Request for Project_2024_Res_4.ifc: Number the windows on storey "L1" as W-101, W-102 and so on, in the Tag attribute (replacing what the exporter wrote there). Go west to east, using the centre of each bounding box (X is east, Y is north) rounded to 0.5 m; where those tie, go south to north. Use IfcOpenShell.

First a look at what the model holds.

```python
import ifcopenshell
import ifcopenshell.util.element
import ifcopenshell.util.placement

model = ifcopenshell.open("Project_2024_Res_4.ifc")
print(model.schema)
storey = next(s for s in model.by_type("IfcBuildingStorey") if s.Name == "L1")
windows = [e for e in ifcopenshell.util.element.get_decomposition(storey) if e.is_a("IfcWindow")]
for e in sorted(windows, key=lambda e: e.id()):
    origin = ifcopenshell.util.placement.get_local_placement(e.ObjectPlacement)[:3, 3]
    print(e.id(), e.Tag, e.Name, origin.round(2) + 0.0, sep=" | ")
```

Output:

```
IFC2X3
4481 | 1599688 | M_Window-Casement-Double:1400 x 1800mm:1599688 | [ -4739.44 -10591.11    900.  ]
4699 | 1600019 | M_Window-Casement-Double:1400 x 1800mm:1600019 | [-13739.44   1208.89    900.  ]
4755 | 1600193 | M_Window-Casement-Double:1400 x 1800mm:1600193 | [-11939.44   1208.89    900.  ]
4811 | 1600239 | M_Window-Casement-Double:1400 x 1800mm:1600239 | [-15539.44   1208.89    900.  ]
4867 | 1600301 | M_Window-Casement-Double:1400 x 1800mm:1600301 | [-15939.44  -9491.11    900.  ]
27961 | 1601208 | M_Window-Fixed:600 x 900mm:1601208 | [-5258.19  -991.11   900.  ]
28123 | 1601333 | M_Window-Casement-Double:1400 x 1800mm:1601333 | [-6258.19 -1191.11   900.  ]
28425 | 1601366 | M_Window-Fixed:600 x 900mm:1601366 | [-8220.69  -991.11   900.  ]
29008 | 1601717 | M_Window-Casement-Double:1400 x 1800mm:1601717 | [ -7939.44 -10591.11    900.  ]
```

```python
import ifcopenshell
import ifcopenshell.geom
import ifcopenshell.util.element
import ifcopenshell.util.shape

model = ifcopenshell.open("Project_2024_Res_4.ifc")
settings = ifcopenshell.geom.settings()
settings.set("use-world-coords", True)


def centre(element):
    shape = ifcopenshell.geom.create_shape(settings, element)
    return ifcopenshell.util.shape.get_bbox_centroid(shape.geometry)


storey = next(s for s in model.by_type("IfcBuildingStorey") if s.Name == "L1")
windows = [e for e in ifcopenshell.util.element.get_decomposition(storey) if e.is_a("IfcWindow")]

# Insertion points can sit at a corner or the storey origin, so sort by the geometry (in metres).
centres = {e: centre(e) for e in windows}
windows.sort(key=lambda e: (round(centres[e][0] / 0.5), centres[e][1]))

for i, e in enumerate(windows, start=1):
    number = f"W-1{i:02d}"
    e.Tag = number
    print(e.id(), number)

model.write("Project_2024_Res_4_updated.ifc")
```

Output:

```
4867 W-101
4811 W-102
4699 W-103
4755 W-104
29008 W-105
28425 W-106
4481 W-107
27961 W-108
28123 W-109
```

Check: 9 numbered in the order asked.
